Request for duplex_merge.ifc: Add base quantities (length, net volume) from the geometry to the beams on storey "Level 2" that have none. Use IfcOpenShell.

First a look at what the model holds.

```python
import ifcopenshell
import ifcopenshell.util.element
import ifcopenshell.util.unit

model = ifcopenshell.open("duplex_merge.ifc")
print(model.schema)
for unit_type in ("LENGTHUNIT", "AREAUNIT", "VOLUMEUNIT"):
    print(unit_type, ifcopenshell.util.unit.calculate_unit_scale(model, unit_type))
storey = next(s for s in model.by_type("IfcBuildingStorey") if s.Name == "Level 2")
beams = [e for e in ifcopenshell.util.element.get_decomposition(storey) if e.is_a("IfcBeam")]
for e in sorted(beams, key=lambda e: e.id()):
    print(e.id(), e.is_a(), e.Name, list(ifcopenshell.util.element.get_psets(e, qtos_only=True)), sep=" | ")
```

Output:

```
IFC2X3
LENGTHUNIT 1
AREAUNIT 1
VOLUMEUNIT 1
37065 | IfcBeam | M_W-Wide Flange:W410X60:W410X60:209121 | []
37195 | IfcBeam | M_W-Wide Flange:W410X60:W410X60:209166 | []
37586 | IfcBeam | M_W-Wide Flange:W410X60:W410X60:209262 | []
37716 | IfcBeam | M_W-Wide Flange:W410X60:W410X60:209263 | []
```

```python
import ifcopenshell
import ifcopenshell.api.pset
import ifcopenshell.geom
import ifcopenshell.util.element
import ifcopenshell.util.shape
import ifcopenshell.util.unit

model = ifcopenshell.open("duplex_merge.ifc")
unit_scale = ifcopenshell.util.unit.calculate_unit_scale(model)
volume_scale = ifcopenshell.util.unit.calculate_unit_scale(model, "VOLUMEUNIT")
settings = ifcopenshell.geom.settings()

storey = next(s for s in model.by_type("IfcBuildingStorey") if s.Name == "Level 2")
beams = [e for e in ifcopenshell.util.element.get_decomposition(storey) if e.is_a("IfcBeam")]

for e in sorted(beams, key=lambda e: e.id()):
    if ifcopenshell.util.element.get_psets(e, qtos_only=True, should_inherit=False):
        continue
    # Geometry comes back in metres, in the element's own axes.
    shape = ifcopenshell.geom.create_shape(settings, e)
    values = {
        "Length": ifcopenshell.util.shape.get_max_xyz(shape.geometry) / unit_scale,
        "NetVolume": ifcopenshell.util.shape.get_volume(shape.geometry) / volume_scale,
    }
    qto = ifcopenshell.api.pset.add_qto(model, product=e, name="BaseQuantities")
    ifcopenshell.api.pset.edit_qto(model, qto=qto, properties=values)
    print(e.id(), {k: round(v, 3) for k, v in values.items()})

model.write("duplex_merge_updated.ifc")
```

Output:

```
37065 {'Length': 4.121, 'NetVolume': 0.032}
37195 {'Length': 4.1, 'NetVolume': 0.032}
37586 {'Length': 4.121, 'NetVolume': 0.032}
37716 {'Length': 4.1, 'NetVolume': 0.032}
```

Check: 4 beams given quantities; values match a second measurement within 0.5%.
